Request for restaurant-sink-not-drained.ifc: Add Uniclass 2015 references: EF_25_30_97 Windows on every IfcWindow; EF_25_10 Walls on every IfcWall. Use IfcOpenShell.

First a look at what the model holds.

```python
import ifcopenshell

model = ifcopenshell.open("restaurant-sink-not-drained.ifc")
print(model.schema)
print("classifications:", [c.Name for c in model.by_type("IfcClassification")])
for ifc_class in ("IfcDoor", "IfcRoof", "IfcStair", "IfcWall", "IfcWindow"):
    print(ifc_class, len(model.by_type(ifc_class)))
```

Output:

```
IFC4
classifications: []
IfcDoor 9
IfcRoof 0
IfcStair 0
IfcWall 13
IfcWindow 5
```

```python
import ifcopenshell
import ifcopenshell.api.classification

model = ifcopenshell.open("restaurant-sink-not-drained.ifc")

system = ifcopenshell.api.classification.add_classification(model, classification="Uniclass 2015")

codes = {
    "IfcWindow": ("EF_25_30_97", "Windows"),
    "IfcWall": ("EF_25_10", "Walls"),
}
for ifc_class, (code, name) in codes.items():
    products = model.by_type(ifc_class)
    ifcopenshell.api.classification.add_reference(
        model, products=products, classification=system, identification=code, name=name
    )
    print(code, len(products))

model.write("restaurant-sink-not-drained_v2.ifc")
```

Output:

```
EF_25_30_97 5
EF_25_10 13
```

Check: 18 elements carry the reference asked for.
